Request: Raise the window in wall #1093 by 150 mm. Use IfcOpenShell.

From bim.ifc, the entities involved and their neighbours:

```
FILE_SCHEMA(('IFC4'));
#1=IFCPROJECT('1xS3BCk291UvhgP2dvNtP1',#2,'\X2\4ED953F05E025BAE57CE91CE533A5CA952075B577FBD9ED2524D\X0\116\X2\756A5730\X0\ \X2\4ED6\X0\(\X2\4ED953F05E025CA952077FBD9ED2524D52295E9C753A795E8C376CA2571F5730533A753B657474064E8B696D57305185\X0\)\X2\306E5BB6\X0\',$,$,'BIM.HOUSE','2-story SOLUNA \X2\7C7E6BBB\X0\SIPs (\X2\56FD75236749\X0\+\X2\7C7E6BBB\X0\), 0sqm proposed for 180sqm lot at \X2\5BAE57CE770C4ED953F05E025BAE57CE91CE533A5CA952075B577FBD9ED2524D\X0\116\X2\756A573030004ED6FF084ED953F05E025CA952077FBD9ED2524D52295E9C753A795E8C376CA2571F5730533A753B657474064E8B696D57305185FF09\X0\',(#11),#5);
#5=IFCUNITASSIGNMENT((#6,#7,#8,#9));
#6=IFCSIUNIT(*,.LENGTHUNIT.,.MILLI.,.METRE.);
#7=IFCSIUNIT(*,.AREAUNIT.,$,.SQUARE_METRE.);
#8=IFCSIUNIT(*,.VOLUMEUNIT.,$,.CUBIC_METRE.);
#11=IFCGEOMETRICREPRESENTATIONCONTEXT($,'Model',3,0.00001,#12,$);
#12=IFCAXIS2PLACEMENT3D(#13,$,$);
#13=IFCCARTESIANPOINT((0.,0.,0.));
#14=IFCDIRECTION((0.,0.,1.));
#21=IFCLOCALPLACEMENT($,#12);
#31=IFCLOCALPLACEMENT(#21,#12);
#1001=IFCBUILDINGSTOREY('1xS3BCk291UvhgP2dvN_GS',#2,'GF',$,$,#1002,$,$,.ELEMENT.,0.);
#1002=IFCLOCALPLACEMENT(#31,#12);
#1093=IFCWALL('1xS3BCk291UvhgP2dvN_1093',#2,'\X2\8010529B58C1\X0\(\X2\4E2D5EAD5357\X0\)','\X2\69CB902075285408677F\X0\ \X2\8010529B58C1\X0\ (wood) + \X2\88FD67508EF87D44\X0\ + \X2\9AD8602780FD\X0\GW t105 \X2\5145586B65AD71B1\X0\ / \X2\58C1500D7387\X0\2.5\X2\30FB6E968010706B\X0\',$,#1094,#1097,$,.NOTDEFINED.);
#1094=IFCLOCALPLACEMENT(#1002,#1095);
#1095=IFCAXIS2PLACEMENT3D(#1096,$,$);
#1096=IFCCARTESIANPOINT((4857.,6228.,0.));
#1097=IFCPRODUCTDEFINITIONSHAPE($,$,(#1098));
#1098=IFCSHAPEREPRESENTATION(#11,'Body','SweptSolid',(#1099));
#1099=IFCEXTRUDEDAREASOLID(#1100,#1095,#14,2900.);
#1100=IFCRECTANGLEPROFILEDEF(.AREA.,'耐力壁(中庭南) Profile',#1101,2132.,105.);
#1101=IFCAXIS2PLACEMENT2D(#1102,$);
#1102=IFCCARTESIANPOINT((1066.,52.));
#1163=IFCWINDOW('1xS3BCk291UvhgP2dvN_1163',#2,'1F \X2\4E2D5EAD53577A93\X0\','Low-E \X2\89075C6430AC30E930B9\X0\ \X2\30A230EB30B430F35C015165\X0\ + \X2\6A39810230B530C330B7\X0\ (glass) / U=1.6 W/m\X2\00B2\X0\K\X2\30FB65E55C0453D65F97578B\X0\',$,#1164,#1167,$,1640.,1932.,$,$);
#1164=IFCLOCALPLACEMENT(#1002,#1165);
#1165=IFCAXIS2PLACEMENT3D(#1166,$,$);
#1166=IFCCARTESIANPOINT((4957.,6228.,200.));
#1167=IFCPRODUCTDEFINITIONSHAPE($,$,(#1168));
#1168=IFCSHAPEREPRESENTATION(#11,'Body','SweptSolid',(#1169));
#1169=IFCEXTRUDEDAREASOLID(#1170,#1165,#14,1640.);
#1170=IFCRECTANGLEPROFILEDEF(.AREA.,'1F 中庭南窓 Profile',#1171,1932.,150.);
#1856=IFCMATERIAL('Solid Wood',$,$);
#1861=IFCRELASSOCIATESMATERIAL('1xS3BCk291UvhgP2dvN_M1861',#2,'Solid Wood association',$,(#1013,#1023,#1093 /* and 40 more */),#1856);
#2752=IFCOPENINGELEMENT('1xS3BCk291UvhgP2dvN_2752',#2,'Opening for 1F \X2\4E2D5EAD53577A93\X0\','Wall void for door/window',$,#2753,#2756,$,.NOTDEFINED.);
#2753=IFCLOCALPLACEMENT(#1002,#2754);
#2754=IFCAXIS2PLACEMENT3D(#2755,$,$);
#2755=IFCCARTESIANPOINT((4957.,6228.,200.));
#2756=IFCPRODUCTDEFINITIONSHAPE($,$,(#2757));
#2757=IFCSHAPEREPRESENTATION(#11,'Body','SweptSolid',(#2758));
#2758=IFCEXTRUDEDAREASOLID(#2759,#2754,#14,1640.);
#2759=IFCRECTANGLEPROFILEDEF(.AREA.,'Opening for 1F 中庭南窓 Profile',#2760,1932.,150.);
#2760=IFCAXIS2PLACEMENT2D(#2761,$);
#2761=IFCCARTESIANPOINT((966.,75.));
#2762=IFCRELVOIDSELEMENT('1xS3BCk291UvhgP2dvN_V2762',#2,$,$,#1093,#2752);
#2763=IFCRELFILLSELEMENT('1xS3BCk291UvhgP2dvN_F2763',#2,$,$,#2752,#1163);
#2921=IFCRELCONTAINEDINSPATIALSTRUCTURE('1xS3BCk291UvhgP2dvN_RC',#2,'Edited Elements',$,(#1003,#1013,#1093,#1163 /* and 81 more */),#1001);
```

```python
import numpy as np
import ifcopenshell
import ifcopenshell.api.geometry
import ifcopenshell.util.placement
import ifcopenshell.util.unit

model = ifcopenshell.open("bim.ifc")
unit_scale = ifcopenshell.util.unit.calculate_unit_scale(model)

window = model.by_guid("1xS3BCk291UvhgP2dvN_1163")
opening = window.FillsVoids[0].RelatingOpeningElement
dz = 0.15 / unit_scale

shift = np.array([0.0, 0.0, dz])
# The window is not placed relative to its opening, so move both.
for product in (opening, window):
    matrix = ifcopenshell.util.placement.get_local_placement(product.ObjectPlacement)
    matrix[:3, 3] += shift
    ifcopenshell.api.geometry.edit_object_placement(model, product=product, matrix=matrix, is_si=False)

print(f"moved by {dz * unit_scale:+.3f} m")

model.write("bim_updated.ifc")
```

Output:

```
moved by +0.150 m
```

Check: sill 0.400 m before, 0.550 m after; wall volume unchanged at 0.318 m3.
